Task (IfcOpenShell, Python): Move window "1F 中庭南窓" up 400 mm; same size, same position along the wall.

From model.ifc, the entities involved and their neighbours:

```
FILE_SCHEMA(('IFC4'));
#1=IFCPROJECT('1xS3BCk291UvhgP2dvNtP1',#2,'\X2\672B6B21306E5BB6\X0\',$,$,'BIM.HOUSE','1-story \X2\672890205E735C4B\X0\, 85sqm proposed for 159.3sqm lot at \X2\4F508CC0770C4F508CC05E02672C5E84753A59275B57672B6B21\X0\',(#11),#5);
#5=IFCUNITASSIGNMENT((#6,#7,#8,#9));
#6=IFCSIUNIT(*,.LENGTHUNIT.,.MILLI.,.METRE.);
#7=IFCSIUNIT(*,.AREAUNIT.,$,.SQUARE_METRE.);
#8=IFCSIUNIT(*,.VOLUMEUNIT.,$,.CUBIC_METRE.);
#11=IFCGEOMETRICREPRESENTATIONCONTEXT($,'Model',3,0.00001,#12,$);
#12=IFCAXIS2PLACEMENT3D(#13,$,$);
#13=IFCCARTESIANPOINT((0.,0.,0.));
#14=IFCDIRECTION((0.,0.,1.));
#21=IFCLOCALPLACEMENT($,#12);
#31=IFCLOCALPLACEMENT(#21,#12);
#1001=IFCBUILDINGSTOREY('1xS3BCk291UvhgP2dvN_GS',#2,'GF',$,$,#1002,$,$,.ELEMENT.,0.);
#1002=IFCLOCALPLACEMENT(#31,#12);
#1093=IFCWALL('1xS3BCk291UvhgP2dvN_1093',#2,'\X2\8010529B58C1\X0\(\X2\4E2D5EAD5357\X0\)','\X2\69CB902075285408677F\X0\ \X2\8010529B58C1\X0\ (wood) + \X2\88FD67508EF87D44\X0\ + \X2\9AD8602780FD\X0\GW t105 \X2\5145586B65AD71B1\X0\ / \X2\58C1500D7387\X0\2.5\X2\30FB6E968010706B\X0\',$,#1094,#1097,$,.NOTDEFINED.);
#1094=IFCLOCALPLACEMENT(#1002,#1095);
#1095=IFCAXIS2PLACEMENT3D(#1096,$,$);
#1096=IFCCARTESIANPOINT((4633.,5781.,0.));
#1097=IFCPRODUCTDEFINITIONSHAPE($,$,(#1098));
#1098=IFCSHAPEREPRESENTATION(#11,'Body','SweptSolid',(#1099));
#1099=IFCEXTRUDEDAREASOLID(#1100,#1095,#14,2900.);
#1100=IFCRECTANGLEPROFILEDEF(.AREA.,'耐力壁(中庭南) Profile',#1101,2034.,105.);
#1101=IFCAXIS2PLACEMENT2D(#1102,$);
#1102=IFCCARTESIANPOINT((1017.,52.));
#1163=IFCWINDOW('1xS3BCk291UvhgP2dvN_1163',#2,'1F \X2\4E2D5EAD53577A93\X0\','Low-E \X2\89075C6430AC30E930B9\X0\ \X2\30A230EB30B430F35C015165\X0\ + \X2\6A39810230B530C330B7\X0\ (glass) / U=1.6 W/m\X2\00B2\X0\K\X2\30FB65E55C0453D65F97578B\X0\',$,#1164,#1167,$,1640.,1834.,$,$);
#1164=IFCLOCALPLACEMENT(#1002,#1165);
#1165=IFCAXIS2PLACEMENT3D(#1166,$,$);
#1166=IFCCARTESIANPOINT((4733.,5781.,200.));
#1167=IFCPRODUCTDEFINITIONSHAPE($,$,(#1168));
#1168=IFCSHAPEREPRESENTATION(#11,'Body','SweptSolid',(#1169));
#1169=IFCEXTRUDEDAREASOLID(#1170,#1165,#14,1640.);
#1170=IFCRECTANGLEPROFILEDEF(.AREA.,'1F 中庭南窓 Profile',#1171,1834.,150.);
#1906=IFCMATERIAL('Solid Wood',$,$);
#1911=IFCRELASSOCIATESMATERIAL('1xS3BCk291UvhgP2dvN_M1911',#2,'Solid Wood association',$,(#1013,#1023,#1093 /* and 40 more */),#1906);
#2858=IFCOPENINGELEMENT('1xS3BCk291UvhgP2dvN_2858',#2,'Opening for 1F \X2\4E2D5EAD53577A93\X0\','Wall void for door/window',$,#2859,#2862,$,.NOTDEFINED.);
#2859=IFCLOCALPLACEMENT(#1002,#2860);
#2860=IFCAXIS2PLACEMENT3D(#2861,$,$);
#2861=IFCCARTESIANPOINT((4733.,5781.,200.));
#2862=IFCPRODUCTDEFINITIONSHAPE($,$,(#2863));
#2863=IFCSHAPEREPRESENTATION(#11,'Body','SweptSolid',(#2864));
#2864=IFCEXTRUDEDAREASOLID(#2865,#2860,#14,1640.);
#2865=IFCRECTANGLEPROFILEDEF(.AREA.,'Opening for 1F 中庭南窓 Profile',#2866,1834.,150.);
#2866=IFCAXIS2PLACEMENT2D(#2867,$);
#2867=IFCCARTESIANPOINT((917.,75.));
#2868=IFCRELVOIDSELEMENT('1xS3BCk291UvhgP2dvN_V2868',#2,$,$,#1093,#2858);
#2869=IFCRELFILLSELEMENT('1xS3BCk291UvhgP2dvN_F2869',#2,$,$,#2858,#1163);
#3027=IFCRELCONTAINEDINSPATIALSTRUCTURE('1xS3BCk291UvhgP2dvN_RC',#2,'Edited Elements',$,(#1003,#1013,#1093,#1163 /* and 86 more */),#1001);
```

```python
import numpy as np
import ifcopenshell
import ifcopenshell.api.geometry
import ifcopenshell.util.placement
import ifcopenshell.util.unit

model = ifcopenshell.open("model.ifc")
unit_scale = ifcopenshell.util.unit.calculate_unit_scale(model)

window = model.by_id(1163)
opening = window.FillsVoids[0].RelatingOpeningElement
dz = 0.4 / unit_scale

shift = np.array([0.0, 0.0, dz])
# The window is not placed relative to its opening, so move both.
for product in (opening, window):
    matrix = ifcopenshell.util.placement.get_local_placement(product.ObjectPlacement)
    matrix[:3, 3] += shift
    ifcopenshell.api.geometry.edit_object_placement(model, product=product, matrix=matrix, is_si=False)

print(f"moved by {dz * unit_scale:+.3f} m")

model.write("model-out.ifc")
```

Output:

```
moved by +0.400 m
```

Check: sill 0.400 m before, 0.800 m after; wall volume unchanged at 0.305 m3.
